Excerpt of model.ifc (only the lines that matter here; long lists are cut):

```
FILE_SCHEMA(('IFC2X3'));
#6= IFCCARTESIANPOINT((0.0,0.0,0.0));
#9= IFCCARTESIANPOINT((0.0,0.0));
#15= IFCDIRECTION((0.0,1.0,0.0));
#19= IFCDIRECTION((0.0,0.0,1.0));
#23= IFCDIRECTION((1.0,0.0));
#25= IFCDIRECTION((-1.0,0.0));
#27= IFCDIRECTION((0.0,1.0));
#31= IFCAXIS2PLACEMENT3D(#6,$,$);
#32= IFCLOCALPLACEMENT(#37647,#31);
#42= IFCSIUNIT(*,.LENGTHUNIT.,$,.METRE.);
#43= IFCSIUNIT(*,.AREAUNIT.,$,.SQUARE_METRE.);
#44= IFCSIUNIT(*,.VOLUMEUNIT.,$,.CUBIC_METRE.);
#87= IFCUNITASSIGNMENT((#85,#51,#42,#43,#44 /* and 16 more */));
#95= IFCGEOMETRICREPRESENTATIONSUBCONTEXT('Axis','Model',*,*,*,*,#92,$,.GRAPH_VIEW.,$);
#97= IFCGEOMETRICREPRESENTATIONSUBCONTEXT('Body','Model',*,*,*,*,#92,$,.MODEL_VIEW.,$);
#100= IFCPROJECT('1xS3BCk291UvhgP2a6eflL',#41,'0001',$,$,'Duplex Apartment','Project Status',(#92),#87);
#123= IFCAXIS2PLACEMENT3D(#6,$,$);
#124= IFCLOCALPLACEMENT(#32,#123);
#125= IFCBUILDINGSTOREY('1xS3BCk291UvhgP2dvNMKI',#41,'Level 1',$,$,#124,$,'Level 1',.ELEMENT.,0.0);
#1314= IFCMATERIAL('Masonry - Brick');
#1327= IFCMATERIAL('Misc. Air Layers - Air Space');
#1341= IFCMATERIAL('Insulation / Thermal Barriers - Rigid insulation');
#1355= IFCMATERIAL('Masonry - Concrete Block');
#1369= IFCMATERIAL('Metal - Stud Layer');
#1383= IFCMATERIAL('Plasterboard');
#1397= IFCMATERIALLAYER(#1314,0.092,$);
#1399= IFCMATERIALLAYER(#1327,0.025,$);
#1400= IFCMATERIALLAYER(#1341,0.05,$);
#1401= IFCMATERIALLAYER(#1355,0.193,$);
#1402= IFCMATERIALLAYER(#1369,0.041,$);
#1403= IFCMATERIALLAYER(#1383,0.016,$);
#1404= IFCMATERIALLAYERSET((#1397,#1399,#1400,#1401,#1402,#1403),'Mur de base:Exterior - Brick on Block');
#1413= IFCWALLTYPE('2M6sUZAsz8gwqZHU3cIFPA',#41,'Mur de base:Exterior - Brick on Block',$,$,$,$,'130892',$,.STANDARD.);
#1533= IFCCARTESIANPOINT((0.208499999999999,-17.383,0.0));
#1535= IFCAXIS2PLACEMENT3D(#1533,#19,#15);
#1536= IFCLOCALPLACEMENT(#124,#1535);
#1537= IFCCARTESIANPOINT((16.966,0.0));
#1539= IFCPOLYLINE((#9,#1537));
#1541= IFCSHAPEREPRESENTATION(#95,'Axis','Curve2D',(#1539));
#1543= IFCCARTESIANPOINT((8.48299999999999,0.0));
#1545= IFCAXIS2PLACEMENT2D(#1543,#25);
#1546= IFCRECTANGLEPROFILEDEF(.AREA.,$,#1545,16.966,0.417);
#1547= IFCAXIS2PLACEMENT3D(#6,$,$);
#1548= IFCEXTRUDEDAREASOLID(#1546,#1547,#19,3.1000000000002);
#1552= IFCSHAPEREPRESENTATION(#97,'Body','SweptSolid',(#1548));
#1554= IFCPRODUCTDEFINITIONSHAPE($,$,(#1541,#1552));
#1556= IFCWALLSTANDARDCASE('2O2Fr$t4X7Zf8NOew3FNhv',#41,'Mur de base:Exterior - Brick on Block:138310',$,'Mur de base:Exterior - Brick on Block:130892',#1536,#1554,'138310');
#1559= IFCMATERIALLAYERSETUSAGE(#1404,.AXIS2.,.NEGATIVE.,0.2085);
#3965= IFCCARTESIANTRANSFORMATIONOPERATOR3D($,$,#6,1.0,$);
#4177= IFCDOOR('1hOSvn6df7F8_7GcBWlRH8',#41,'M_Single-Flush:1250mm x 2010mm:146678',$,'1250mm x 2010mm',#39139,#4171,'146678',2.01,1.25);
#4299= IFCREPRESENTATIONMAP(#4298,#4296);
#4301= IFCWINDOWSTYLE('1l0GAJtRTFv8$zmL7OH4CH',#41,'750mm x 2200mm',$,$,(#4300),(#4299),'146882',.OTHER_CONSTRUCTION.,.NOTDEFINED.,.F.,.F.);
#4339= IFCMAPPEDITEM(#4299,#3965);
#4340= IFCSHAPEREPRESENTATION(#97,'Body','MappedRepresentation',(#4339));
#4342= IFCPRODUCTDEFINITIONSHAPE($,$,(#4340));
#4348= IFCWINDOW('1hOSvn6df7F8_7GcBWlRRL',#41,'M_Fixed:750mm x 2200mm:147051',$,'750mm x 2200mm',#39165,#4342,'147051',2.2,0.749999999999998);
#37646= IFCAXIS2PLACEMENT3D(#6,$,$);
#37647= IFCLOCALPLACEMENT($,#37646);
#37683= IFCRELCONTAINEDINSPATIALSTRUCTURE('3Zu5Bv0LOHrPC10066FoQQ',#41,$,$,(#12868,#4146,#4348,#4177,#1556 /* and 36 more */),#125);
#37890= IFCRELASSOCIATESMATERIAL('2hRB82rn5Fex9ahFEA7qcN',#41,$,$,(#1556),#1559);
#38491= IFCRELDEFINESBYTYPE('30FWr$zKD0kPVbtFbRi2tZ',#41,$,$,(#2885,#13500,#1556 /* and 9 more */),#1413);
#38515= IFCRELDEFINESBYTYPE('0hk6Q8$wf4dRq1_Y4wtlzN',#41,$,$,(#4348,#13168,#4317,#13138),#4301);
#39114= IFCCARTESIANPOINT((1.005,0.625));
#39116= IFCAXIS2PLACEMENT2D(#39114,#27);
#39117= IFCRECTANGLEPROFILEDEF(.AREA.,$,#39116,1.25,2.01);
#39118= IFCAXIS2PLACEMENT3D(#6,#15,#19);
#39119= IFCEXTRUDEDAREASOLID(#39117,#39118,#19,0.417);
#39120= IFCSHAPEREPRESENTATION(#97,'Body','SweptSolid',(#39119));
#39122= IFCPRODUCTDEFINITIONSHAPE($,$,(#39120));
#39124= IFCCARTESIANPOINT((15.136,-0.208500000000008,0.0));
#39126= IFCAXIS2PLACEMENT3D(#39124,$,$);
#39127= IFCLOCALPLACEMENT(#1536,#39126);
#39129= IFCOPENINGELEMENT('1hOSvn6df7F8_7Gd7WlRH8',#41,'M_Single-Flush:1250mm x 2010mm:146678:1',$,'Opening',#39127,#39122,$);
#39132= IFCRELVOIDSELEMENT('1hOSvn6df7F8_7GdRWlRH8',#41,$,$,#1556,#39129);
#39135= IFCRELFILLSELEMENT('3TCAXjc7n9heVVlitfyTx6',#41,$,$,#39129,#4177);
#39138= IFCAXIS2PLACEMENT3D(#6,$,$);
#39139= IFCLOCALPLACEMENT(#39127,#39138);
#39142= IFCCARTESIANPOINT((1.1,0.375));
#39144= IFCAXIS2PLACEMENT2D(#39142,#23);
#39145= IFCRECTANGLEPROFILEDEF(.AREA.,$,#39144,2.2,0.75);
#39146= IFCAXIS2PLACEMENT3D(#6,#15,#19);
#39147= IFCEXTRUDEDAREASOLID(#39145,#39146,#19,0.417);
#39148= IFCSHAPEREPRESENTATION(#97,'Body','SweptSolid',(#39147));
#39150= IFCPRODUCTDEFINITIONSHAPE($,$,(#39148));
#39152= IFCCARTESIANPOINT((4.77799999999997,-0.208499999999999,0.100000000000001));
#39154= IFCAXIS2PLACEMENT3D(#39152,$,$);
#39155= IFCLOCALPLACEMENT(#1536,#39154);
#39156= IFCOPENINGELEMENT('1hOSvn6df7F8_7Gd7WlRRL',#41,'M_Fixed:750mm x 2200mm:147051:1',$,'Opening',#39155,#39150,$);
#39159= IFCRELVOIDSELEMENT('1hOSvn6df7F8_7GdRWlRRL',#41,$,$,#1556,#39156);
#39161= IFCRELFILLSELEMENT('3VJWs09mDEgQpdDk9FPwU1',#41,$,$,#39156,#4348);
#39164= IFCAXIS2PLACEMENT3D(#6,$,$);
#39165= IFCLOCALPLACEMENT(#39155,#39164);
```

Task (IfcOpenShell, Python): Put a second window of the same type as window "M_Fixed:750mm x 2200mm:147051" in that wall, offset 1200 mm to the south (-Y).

```python
import ifcopenshell
import ifcopenshell.api.feature
import ifcopenshell.api.geometry
import ifcopenshell.api.root
import ifcopenshell.geom
import ifcopenshell.util.element
import ifcopenshell.util.placement
import ifcopenshell.util.shape
import ifcopenshell.util.unit

model = ifcopenshell.open("model.ifc")
unit_scale = ifcopenshell.util.unit.calculate_unit_scale(model)
settings = ifcopenshell.geom.settings()


def volume(element):
    """Net volume in cubic metres, openings subtracted."""
    shape = ifcopenshell.geom.create_shape(settings, element)
    return ifcopenshell.util.shape.get_volume(shape.geometry)


def reuse_history(source, copy):
    """copy_class also copies each property set's owner history, people and application; keep the originals."""
    for rel in copy.IsDefinedBy:
        if rel.is_a("IfcRelDefinesByProperties") and (history := rel.RelatingPropertyDefinition.OwnerHistory):
            rel.RelatingPropertyDefinition.OwnerHistory = source.OwnerHistory
            ifcopenshell.util.element.remove_deep2(model, history)


window = model.by_id(4348)
opening = window.FillsVoids[0].RelatingOpeningElement
wall = opening.VoidsElements[0].RelatingBuildingElement
before = volume(wall)
shift = ifcopenshell.util.placement.get_local_placement(wall.ObjectPlacement)[:3, 0] * -1.2 / unit_scale

# copy_class copies the void relationship, type, container and properties, but no geometry.
new_opening = ifcopenshell.api.root.copy_class(model, product=opening)
new_opening.Representation = ifcopenshell.util.element.copy_deep(
    model, opening.Representation, exclude=["IfcGeometricRepresentationContext", "IfcRepresentationMap"]
)
new_opening.Name = "M_Fixed:750mm x 2200mm"
new_window = ifcopenshell.api.root.copy_class(model, product=window)
new_window.Representation = ifcopenshell.util.element.copy_deep(
    model, window.Representation, exclude=["IfcGeometricRepresentationContext", "IfcRepresentationMap"]
)
new_window.Name = "M_Fixed:750mm x 2200mm"
new_window.Tag = None
reuse_history(window, new_window)
fills = ifcopenshell.api.feature.add_filling(model, opening=new_opening, element=new_window)
fills.OwnerHistory = new_window.OwnerHistory  # required in IFC2X3

for old, new in ((opening, new_opening), (window, new_window)):
    matrix = ifcopenshell.util.placement.get_local_placement(old.ObjectPlacement)
    matrix[:3, 3] += shift
    ifcopenshell.api.geometry.edit_object_placement(model, product=new, matrix=matrix, is_si=False)

after = volume(wall)

print(f"wall volume {before:.3f} -> {after:.3f} m3")

model.write("model_updated.ifc")
```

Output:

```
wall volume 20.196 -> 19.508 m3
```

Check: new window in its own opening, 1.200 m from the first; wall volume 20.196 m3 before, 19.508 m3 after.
